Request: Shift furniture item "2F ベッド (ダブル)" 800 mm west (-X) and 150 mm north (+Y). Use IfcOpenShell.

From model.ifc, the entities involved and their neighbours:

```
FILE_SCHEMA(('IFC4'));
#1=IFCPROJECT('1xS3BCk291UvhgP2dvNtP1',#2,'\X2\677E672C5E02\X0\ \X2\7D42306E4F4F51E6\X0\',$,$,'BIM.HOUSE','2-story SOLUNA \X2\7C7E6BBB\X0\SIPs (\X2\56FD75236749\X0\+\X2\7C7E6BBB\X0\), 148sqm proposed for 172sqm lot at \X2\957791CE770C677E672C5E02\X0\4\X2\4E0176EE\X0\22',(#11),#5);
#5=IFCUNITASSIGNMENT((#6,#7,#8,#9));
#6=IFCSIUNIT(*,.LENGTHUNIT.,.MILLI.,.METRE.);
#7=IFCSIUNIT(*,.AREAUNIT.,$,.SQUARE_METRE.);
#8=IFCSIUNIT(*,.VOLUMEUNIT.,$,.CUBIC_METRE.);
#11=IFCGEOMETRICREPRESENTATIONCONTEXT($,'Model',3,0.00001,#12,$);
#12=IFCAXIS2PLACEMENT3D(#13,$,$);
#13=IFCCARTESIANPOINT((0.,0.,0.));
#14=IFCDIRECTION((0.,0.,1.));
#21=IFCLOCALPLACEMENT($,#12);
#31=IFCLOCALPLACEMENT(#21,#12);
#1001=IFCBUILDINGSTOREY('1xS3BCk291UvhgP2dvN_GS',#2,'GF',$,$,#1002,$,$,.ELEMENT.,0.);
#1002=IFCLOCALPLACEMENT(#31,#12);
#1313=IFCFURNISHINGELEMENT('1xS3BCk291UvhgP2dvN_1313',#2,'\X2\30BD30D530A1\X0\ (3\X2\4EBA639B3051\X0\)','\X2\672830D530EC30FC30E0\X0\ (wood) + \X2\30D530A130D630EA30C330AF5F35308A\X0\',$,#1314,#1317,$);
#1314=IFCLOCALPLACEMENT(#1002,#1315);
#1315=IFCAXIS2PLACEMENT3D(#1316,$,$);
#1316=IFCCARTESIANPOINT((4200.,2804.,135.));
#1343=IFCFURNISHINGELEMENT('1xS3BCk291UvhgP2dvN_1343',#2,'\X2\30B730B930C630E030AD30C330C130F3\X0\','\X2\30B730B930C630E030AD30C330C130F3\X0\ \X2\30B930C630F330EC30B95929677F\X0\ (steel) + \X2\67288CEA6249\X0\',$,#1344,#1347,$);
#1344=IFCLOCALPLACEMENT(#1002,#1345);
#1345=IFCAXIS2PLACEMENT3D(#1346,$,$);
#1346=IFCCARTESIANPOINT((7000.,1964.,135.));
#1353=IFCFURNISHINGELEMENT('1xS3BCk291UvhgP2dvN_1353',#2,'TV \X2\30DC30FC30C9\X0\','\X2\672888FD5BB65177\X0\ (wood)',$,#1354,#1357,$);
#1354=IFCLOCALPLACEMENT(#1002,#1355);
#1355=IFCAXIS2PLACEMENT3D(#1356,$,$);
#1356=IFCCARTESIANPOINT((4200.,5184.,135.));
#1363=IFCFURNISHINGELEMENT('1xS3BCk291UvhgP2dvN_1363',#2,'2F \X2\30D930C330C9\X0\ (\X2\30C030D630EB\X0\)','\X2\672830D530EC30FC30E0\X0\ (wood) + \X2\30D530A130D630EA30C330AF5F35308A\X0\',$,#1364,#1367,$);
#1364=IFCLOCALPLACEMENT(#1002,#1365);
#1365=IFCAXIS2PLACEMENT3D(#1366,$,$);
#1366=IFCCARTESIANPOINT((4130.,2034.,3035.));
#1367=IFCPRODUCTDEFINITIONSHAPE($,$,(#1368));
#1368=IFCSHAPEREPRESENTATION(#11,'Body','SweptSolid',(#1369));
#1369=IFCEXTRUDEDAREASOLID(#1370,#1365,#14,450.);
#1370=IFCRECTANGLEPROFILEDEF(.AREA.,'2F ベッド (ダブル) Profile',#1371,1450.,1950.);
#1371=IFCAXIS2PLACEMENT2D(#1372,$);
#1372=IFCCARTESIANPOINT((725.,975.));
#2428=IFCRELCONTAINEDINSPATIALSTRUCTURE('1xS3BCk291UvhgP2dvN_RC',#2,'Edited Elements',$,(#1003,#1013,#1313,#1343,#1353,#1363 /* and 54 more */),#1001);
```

```python
import ifcopenshell
import ifcopenshell.api.geometry
import ifcopenshell.util.placement
import ifcopenshell.util.unit

model = ifcopenshell.open("model.ifc")
unit_scale = ifcopenshell.util.unit.calculate_unit_scale(model)

item = model.by_guid("1xS3BCk291UvhgP2dvN_1363")
matrix = ifcopenshell.util.placement.get_local_placement(item.ObjectPlacement)
matrix[0, 3] -= 0.8 / unit_scale
matrix[1, 3] += 0.15 / unit_scale
ifcopenshell.api.geometry.edit_object_placement(model, product=item, matrix=matrix, is_si=False)

print(ifcopenshell.util.placement.get_local_placement(item.ObjectPlacement).round(3) + 0.0)

model.write("model_v2.ifc")
```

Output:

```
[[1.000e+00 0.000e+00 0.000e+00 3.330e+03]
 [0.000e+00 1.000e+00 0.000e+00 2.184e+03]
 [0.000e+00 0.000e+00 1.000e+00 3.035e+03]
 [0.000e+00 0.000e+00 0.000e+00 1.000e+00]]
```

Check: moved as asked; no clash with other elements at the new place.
